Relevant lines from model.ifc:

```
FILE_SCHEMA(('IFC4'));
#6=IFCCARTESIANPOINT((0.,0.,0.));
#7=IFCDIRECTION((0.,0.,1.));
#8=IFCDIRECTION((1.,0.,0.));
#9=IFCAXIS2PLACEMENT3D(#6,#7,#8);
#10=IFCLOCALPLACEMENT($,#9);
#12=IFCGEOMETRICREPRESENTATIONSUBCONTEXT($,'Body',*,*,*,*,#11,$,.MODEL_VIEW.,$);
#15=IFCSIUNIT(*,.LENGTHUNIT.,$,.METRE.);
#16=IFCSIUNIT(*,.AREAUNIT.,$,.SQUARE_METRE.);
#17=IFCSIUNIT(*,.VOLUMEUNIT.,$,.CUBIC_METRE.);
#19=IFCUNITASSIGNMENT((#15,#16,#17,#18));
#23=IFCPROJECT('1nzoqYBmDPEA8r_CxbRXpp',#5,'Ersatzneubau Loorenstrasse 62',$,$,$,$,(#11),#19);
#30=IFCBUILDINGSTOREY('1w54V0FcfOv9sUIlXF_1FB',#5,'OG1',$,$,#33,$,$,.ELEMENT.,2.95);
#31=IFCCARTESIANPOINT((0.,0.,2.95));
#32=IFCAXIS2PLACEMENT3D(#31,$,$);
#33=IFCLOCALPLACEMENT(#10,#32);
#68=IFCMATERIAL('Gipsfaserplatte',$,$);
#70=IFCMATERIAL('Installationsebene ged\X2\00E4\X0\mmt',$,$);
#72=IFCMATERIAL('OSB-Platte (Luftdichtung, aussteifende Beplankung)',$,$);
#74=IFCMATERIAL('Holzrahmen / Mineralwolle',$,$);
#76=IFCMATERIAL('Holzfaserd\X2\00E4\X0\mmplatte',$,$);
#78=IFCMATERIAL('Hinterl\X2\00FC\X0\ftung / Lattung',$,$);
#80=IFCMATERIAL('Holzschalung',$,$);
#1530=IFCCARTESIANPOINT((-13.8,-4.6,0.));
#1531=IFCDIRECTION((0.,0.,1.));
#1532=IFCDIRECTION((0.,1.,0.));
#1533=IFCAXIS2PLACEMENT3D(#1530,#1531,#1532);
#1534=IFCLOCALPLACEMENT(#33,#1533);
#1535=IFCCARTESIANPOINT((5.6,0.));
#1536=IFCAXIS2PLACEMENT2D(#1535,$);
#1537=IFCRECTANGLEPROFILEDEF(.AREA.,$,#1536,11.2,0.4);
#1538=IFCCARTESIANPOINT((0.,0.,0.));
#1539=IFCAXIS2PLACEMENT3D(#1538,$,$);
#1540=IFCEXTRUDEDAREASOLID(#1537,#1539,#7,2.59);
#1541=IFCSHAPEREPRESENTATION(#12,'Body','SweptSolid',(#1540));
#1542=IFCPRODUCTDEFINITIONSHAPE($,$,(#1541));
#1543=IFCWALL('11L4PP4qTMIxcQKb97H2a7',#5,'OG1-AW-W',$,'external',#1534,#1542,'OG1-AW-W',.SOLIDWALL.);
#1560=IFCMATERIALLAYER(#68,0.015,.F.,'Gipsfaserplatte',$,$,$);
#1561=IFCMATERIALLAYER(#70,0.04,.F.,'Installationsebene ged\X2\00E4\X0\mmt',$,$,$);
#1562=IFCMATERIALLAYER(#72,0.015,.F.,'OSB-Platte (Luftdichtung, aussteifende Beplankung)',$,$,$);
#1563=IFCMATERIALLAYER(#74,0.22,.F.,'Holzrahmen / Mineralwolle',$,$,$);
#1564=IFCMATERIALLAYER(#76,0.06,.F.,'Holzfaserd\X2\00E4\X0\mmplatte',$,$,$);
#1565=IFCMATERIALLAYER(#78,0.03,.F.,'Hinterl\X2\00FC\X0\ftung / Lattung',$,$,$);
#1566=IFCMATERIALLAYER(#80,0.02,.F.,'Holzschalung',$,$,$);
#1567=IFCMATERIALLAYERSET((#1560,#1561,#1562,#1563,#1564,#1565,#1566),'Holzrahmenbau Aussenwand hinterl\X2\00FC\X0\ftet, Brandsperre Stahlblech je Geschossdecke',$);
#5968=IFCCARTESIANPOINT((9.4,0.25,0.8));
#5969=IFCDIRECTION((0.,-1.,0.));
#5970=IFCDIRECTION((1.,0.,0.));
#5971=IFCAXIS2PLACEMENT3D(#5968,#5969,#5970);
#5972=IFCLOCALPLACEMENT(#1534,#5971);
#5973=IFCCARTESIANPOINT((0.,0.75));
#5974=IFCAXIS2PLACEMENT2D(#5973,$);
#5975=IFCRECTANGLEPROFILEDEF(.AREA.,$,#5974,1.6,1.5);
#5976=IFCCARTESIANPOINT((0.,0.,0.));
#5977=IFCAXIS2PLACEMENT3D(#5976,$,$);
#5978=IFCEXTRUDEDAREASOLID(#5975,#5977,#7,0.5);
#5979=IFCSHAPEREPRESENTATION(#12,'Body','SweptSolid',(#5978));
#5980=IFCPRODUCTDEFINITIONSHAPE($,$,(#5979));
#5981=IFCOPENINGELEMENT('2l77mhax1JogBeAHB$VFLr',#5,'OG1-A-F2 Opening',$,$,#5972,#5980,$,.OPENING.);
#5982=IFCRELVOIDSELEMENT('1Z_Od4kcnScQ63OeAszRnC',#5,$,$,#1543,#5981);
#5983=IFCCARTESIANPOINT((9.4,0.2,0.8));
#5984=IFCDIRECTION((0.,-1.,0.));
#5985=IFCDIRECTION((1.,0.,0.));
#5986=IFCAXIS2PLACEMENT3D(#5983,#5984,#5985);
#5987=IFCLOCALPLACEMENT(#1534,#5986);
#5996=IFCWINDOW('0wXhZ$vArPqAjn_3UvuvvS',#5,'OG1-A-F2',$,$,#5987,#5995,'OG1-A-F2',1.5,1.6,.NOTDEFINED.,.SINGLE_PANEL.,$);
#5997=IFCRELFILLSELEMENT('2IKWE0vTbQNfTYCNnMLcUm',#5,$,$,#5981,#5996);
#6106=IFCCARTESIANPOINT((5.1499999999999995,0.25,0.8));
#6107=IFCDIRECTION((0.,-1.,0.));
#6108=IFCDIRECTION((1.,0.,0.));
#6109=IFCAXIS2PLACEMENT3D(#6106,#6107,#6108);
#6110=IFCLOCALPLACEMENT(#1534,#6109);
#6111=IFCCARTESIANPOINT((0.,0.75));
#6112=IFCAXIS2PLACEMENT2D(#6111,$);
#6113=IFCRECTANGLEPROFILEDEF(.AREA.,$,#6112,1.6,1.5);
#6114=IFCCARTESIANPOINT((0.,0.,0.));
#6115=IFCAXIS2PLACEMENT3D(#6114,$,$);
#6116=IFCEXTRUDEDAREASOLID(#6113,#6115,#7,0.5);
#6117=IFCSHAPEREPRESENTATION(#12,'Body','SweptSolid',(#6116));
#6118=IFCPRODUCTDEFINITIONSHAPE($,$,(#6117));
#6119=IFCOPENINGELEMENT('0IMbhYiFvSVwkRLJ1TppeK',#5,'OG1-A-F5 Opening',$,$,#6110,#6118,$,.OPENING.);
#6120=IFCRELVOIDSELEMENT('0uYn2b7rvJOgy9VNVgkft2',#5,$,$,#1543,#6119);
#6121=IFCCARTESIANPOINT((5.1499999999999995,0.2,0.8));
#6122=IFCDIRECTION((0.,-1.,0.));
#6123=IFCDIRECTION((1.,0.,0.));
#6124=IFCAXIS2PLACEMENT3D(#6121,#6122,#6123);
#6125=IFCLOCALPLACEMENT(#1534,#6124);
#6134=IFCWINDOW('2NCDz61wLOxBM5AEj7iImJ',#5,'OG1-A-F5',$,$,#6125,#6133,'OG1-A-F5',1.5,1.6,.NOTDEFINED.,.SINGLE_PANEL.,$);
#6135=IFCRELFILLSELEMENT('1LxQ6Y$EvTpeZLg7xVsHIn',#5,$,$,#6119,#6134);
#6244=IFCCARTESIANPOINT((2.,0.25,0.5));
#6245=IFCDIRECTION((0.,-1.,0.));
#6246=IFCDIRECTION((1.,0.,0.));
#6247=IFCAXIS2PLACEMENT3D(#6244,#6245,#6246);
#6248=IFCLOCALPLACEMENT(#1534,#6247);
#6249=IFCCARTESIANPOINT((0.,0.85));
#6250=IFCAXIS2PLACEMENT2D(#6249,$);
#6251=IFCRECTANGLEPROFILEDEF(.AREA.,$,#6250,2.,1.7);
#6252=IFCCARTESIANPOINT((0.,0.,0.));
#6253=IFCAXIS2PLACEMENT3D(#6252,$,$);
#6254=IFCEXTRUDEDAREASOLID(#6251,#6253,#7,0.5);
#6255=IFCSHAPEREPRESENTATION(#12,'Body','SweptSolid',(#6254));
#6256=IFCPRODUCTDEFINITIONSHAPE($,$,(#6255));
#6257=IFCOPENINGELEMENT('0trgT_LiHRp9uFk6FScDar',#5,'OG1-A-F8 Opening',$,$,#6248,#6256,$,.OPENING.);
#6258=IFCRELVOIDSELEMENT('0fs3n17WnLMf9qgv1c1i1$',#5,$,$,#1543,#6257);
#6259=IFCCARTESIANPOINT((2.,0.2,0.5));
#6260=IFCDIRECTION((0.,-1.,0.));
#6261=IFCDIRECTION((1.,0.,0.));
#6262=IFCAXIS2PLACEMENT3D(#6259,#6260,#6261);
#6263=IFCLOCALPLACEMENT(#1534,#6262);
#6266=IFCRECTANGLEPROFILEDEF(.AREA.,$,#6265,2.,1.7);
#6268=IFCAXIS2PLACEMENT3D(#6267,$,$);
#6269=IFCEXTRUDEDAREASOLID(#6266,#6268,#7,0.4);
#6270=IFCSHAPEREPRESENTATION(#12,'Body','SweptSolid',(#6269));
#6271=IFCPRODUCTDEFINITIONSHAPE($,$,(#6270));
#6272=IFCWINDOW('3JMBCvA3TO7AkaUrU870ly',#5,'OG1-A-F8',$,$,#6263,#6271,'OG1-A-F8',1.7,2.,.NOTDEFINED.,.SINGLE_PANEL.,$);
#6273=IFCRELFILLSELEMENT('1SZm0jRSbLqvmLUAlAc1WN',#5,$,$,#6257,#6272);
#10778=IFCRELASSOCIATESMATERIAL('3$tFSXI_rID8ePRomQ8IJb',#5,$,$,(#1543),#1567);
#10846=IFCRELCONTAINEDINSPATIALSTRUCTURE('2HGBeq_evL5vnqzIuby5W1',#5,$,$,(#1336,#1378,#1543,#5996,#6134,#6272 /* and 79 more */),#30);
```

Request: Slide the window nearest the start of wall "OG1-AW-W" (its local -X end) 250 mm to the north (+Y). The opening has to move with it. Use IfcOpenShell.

```python
import ifcopenshell
import ifcopenshell.api.geometry
import ifcopenshell.util.placement
import ifcopenshell.util.unit

model = ifcopenshell.open("model.ifc")
unit_scale = ifcopenshell.util.unit.calculate_unit_scale(model)

window = model.by_guid("3JMBCvA3TO7AkaUrU870ly")
opening = window.FillsVoids[0].RelatingOpeningElement
wall = opening.VoidsElements[0].RelatingBuildingElement

wall_matrix = ifcopenshell.util.placement.get_local_placement(wall.ObjectPlacement)
shift = wall_matrix[:3, 0] * 0.25 / unit_scale
before = ifcopenshell.util.placement.get_local_placement(window.ObjectPlacement)[:3, 3].copy()

# The window is not placed relative to its opening, so move both.
for product in (opening, window):
    matrix = ifcopenshell.util.placement.get_local_placement(product.ObjectPlacement)
    matrix[:3, 3] += shift
    ifcopenshell.api.geometry.edit_object_placement(model, product=product, matrix=matrix, is_si=False)

after = ifcopenshell.util.placement.get_local_placement(window.ObjectPlacement)[:3, 3]
print("window moved by", (after - before).round(3) + 0.0)

model.write("model_updated.ifc")
```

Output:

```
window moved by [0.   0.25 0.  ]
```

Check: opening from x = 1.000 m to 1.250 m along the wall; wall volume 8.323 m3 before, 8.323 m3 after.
